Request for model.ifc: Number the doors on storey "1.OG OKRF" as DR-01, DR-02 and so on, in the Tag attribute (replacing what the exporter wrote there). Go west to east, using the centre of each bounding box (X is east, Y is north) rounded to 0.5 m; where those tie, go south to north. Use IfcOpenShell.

First a look at what the model holds.

```python
import ifcopenshell
import ifcopenshell.util.element
import ifcopenshell.util.placement

model = ifcopenshell.open("model.ifc")
print(model.schema)
storey = next(s for s in model.by_type("IfcBuildingStorey") if s.Name == "1.OG OKRF")
doors = [e for e in ifcopenshell.util.element.get_decomposition(storey) if e.is_a("IfcDoor")]
for e in sorted(doors, key=lambda e: e.id()):
    origin = ifcopenshell.util.placement.get_local_placement(e.ObjectPlacement)[:3, 3]
    print(e.id(), e.Tag, e.Name, origin.round(2) + 0.0, sep=" | ")
```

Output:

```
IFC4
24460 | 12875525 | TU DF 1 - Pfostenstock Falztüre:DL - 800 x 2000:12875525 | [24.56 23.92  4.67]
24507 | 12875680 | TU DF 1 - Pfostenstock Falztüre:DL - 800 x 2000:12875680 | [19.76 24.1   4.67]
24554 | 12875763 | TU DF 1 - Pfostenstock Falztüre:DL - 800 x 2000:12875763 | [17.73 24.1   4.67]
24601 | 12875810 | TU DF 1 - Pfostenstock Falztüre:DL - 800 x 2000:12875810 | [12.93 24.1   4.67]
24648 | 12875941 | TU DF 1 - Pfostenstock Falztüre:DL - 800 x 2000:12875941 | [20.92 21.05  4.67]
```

```python
import ifcopenshell
import ifcopenshell.geom
import ifcopenshell.util.element
import ifcopenshell.util.shape

model = ifcopenshell.open("model.ifc")
settings = ifcopenshell.geom.settings()
settings.set("use-world-coords", True)


def centre(element):
    shape = ifcopenshell.geom.create_shape(settings, element)
    return ifcopenshell.util.shape.get_bbox_centroid(shape.geometry)


storey = next(s for s in model.by_type("IfcBuildingStorey") if s.Name == "1.OG OKRF")
doors = [e for e in ifcopenshell.util.element.get_decomposition(storey) if e.is_a("IfcDoor")]

# Insertion points can sit at a corner or the storey origin, so sort by the geometry (in metres).
centres = {e: centre(e) for e in doors}
doors.sort(key=lambda e: (round(centres[e][0] / 0.5), centres[e][1]))

for i, e in enumerate(doors, start=1):
    number = f"DR-{i:02d}"
    e.Tag = number
    print(e.id(), number)

model.write("model_rev.ifc")
```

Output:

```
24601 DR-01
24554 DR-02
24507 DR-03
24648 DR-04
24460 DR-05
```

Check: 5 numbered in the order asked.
